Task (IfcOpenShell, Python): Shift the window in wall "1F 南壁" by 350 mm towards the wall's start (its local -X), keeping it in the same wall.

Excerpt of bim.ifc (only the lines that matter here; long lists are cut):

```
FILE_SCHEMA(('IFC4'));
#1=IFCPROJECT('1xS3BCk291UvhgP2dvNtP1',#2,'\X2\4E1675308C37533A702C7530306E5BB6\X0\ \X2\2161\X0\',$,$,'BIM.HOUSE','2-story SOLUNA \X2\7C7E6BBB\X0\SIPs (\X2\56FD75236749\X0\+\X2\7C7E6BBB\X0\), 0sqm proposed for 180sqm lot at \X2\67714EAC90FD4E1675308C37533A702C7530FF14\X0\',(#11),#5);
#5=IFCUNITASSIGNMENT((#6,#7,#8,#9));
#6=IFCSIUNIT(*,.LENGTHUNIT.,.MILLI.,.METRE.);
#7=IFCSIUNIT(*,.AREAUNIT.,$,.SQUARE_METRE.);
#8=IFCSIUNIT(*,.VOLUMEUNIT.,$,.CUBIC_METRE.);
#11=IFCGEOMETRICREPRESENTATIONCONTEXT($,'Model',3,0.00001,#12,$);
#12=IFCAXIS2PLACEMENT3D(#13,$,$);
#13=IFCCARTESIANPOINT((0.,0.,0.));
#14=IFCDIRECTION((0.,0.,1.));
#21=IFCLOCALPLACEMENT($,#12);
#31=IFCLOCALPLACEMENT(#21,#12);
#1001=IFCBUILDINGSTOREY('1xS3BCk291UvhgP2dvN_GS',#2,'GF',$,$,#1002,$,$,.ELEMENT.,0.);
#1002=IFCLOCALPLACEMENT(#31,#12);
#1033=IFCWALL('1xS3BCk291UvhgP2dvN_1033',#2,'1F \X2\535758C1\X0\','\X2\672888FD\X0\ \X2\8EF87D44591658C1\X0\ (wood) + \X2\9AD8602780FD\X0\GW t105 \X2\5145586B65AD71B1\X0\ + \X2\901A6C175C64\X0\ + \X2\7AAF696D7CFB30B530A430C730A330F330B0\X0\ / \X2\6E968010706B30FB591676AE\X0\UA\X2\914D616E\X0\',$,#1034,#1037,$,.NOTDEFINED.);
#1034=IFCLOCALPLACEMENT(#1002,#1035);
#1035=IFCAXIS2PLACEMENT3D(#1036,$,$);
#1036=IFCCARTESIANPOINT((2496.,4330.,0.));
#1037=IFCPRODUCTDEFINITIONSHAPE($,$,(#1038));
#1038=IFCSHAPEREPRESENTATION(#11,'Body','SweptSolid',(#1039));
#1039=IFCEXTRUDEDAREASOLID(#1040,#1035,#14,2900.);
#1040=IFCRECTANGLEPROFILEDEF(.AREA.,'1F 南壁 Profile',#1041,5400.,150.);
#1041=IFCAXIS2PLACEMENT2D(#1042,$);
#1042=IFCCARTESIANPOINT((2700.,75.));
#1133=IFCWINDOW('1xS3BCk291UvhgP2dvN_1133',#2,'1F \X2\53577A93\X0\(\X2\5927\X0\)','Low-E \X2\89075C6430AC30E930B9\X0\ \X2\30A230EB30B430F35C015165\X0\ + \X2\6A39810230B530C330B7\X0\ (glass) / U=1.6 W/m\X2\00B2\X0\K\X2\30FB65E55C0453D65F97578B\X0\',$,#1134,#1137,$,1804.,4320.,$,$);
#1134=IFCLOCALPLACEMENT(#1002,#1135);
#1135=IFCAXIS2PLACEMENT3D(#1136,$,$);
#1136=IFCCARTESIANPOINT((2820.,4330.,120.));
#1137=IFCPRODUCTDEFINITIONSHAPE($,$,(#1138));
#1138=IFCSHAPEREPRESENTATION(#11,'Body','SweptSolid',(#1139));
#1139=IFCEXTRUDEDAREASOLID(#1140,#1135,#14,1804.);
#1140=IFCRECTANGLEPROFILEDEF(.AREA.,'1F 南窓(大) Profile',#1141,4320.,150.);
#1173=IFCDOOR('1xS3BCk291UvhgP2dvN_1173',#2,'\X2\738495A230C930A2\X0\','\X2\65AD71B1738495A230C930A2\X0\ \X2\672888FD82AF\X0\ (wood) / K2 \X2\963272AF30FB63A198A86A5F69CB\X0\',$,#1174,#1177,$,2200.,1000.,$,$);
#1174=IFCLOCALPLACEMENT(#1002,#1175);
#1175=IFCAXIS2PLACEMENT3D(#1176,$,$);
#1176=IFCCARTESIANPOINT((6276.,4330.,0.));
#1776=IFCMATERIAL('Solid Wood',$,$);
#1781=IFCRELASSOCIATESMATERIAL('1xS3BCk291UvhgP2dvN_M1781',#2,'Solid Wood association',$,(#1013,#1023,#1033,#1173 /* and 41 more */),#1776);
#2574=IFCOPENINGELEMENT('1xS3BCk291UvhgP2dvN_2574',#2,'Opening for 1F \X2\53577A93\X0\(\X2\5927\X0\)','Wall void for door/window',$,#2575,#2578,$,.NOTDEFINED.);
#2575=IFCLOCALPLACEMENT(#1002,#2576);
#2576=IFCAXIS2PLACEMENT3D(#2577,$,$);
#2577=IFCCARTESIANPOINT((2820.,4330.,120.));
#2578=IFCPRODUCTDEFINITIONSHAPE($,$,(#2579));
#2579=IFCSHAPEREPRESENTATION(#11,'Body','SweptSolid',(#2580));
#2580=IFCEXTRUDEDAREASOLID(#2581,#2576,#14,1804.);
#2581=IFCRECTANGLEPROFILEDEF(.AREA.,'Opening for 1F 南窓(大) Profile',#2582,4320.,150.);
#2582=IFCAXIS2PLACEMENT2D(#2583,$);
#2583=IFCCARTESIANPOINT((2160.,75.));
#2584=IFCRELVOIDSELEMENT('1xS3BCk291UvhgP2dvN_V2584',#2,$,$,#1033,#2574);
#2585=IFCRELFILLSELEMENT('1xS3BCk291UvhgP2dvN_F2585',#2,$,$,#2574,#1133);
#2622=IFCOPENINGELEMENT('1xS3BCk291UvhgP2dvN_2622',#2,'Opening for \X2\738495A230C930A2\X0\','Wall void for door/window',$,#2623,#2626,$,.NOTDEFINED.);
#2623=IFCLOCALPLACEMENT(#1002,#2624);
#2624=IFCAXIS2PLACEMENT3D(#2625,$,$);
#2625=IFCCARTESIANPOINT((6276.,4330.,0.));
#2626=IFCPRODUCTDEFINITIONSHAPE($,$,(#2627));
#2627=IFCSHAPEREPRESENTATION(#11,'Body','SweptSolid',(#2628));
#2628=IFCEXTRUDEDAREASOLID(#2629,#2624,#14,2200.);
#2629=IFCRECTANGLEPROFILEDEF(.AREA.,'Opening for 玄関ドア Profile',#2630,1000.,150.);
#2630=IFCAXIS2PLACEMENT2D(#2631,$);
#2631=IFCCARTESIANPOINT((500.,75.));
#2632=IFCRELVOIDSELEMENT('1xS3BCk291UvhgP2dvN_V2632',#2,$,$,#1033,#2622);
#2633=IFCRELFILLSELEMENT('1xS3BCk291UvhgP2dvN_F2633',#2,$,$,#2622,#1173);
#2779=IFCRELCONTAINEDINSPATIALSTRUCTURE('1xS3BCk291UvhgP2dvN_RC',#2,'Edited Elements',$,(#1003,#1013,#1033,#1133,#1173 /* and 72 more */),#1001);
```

```python
import ifcopenshell
import ifcopenshell.api.geometry
import ifcopenshell.util.placement
import ifcopenshell.util.unit

model = ifcopenshell.open("bim.ifc")
unit_scale = ifcopenshell.util.unit.calculate_unit_scale(model)

window = model.by_guid("1xS3BCk291UvhgP2dvN_1133")
opening = window.FillsVoids[0].RelatingOpeningElement
wall = opening.VoidsElements[0].RelatingBuildingElement

wall_matrix = ifcopenshell.util.placement.get_local_placement(wall.ObjectPlacement)
shift = wall_matrix[:3, 0] * -0.35 / unit_scale
before = ifcopenshell.util.placement.get_local_placement(window.ObjectPlacement)[:3, 3].copy()

# The window is not placed relative to its opening, so move both.
for product in (opening, window):
    matrix = ifcopenshell.util.placement.get_local_placement(product.ObjectPlacement)
    matrix[:3, 3] += shift
    ifcopenshell.api.geometry.edit_object_placement(model, product=product, matrix=matrix, is_si=False)

after = ifcopenshell.util.placement.get_local_placement(window.ObjectPlacement)[:3, 3]
print("window moved by", (after - before).round(3) + 0.0)

model.write("bim_edited.ifc")
```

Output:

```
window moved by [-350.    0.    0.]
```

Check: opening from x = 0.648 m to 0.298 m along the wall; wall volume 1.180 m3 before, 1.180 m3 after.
